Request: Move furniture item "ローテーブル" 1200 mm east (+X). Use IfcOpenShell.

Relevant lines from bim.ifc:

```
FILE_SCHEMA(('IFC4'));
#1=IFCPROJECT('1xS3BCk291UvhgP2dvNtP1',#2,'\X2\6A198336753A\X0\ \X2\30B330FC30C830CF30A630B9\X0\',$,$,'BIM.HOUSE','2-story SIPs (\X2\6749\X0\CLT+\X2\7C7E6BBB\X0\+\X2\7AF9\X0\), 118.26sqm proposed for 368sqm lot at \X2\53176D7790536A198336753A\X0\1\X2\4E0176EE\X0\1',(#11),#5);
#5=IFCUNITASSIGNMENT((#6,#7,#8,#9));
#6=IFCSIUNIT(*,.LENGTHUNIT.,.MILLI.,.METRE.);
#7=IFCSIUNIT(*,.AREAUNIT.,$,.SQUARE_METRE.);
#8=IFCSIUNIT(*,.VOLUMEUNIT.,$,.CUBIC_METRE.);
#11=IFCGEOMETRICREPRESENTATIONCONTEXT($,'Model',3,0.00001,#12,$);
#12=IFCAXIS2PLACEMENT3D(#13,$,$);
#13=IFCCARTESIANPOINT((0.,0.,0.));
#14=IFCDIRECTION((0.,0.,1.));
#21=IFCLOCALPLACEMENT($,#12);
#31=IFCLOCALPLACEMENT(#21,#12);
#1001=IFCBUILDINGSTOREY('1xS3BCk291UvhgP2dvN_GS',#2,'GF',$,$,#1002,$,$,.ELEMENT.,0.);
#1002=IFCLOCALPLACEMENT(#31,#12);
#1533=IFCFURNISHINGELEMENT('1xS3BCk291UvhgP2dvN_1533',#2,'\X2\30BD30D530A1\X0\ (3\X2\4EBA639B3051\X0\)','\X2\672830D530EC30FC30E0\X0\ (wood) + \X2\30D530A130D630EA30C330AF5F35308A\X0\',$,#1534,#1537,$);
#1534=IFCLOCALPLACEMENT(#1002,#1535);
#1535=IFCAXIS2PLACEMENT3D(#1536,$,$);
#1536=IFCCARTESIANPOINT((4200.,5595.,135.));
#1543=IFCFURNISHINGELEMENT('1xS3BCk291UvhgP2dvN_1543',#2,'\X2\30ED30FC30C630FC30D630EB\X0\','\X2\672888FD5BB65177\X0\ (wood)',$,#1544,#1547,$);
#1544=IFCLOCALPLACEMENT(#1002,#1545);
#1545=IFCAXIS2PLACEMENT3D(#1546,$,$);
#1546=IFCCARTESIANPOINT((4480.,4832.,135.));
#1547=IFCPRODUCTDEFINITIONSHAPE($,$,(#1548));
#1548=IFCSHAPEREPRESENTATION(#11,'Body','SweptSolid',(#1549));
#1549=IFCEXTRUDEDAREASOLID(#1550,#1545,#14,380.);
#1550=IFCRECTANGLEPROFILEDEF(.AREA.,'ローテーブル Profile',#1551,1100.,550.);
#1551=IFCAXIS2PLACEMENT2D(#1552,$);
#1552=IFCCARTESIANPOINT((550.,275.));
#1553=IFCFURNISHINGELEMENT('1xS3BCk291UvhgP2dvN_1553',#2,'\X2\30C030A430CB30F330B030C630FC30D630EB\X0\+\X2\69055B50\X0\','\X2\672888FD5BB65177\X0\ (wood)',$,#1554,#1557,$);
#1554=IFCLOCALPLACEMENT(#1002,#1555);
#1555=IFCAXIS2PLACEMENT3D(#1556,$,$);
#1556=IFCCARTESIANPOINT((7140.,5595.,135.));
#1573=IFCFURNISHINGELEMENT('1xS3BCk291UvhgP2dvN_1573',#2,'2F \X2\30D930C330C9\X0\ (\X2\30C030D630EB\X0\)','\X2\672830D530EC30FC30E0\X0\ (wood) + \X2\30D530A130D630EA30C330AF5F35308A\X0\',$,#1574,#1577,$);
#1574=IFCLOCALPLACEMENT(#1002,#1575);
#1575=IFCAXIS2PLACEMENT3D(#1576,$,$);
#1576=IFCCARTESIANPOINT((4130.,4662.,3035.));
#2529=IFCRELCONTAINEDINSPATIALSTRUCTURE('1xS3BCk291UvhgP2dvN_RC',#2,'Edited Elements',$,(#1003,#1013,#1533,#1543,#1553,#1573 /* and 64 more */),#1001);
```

```python
import ifcopenshell
import ifcopenshell.api.geometry
import ifcopenshell.util.placement

model = ifcopenshell.open("bim.ifc")

item = model.by_guid("1xS3BCk291UvhgP2dvN_1543")
matrix = ifcopenshell.util.placement.get_local_placement(item.ObjectPlacement)
matrix[0, 3] += 1200.0
ifcopenshell.api.geometry.edit_object_placement(model, product=item, matrix=matrix, is_si=False)

print(ifcopenshell.util.placement.get_local_placement(item.ObjectPlacement).round(3) + 0.0)

model.write("bim_updated.ifc")
```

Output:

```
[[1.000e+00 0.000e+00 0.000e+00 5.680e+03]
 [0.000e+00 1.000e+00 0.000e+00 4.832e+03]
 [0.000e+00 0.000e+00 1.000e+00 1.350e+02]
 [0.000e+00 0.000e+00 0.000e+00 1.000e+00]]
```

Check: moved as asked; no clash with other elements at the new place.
